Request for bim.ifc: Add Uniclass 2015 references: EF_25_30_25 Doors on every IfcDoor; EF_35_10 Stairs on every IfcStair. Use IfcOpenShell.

First a look at what the model holds.

```python
import ifcopenshell

model = ifcopenshell.open("bim.ifc")
print(model.schema)
print("classifications:", [c.Name for c in model.by_type("IfcClassification")])
for ifc_class in ("IfcDoor", "IfcRoof", "IfcStair", "IfcWall", "IfcWindow"):
    print(ifc_class, len(model.by_type(ifc_class)))
```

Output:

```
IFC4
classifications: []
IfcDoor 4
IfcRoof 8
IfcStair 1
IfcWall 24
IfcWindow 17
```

```python
import ifcopenshell
import ifcopenshell.api.classification

model = ifcopenshell.open("bim.ifc")

system = ifcopenshell.api.classification.add_classification(model, classification="Uniclass 2015")

codes = {
    "IfcDoor": ("EF_25_30_25", "Doors"),
    "IfcStair": ("EF_35_10", "Stairs"),
}
for ifc_class, (code, name) in codes.items():
    products = model.by_type(ifc_class)
    ifcopenshell.api.classification.add_reference(
        model, products=products, classification=system, identification=code, name=name
    )
    print(code, len(products))

model.write("bim-out.ifc")
```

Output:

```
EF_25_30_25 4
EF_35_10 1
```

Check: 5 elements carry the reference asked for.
